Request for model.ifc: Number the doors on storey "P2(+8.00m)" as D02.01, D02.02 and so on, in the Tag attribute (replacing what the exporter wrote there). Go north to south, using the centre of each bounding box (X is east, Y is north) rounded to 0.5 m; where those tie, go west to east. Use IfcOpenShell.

First a look at what the model holds.

```python
import ifcopenshell
import ifcopenshell.util.element
import ifcopenshell.util.placement

model = ifcopenshell.open("model.ifc")
print(model.schema)
storey = next(s for s in model.by_type("IfcBuildingStorey") if s.Name == "P2(+8.00m)")
doors = [e for e in ifcopenshell.util.element.get_decomposition(storey) if e.is_a("IfcDoor")]
for e in sorted(doors, key=lambda e: e.id()):
    origin = ifcopenshell.util.placement.get_local_placement(e.ObjectPlacement)[:3, 3]
    print(e.id(), e.Tag, e.Name, origin.round(2) + 0.0, sep=" | ")
```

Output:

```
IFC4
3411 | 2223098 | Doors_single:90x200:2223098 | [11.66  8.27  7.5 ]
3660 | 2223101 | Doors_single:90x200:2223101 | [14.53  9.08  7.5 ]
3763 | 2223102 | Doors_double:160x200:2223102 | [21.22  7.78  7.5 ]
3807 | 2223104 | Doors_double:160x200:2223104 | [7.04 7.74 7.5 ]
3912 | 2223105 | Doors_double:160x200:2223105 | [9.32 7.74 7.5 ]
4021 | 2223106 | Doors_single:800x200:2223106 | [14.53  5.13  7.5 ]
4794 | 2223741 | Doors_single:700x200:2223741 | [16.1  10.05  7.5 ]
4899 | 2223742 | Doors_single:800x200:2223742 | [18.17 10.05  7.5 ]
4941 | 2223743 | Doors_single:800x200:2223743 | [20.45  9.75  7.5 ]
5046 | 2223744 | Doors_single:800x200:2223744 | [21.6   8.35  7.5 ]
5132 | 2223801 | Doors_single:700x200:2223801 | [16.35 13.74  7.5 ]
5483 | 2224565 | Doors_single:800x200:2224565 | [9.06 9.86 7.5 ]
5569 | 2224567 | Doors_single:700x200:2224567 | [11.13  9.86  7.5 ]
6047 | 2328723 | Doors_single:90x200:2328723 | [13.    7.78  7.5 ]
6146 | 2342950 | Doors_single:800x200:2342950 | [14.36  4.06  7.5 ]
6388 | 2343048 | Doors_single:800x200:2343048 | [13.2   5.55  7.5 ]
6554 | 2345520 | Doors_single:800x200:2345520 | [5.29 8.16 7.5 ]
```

```python
import ifcopenshell
import ifcopenshell.geom
import ifcopenshell.util.element
import ifcopenshell.util.shape

model = ifcopenshell.open("model.ifc")
settings = ifcopenshell.geom.settings()
settings.set("use-world-coords", True)


def centre(element):
    shape = ifcopenshell.geom.create_shape(settings, element)
    return ifcopenshell.util.shape.get_bbox_centroid(shape.geometry)


storey = next(s for s in model.by_type("IfcBuildingStorey") if s.Name == "P2(+8.00m)")
doors = [e for e in ifcopenshell.util.element.get_decomposition(storey) if e.is_a("IfcDoor")]

# Insertion points can sit at a corner or the storey origin, so sort by the geometry (in metres).
centres = {e: centre(e) for e in doors}
doors.sort(key=lambda e: (-round(centres[e][1] / 0.5), centres[e][0]))

for i, e in enumerate(doors, start=1):
    number = f"D02.{i:02d}"
    e.Tag = number
    print(e.id(), number)

model.write("model_edited.ifc")
```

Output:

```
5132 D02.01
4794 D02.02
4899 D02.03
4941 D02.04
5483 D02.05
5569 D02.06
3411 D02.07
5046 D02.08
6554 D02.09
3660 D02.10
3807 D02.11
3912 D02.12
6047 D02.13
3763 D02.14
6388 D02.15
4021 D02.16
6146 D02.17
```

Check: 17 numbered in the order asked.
